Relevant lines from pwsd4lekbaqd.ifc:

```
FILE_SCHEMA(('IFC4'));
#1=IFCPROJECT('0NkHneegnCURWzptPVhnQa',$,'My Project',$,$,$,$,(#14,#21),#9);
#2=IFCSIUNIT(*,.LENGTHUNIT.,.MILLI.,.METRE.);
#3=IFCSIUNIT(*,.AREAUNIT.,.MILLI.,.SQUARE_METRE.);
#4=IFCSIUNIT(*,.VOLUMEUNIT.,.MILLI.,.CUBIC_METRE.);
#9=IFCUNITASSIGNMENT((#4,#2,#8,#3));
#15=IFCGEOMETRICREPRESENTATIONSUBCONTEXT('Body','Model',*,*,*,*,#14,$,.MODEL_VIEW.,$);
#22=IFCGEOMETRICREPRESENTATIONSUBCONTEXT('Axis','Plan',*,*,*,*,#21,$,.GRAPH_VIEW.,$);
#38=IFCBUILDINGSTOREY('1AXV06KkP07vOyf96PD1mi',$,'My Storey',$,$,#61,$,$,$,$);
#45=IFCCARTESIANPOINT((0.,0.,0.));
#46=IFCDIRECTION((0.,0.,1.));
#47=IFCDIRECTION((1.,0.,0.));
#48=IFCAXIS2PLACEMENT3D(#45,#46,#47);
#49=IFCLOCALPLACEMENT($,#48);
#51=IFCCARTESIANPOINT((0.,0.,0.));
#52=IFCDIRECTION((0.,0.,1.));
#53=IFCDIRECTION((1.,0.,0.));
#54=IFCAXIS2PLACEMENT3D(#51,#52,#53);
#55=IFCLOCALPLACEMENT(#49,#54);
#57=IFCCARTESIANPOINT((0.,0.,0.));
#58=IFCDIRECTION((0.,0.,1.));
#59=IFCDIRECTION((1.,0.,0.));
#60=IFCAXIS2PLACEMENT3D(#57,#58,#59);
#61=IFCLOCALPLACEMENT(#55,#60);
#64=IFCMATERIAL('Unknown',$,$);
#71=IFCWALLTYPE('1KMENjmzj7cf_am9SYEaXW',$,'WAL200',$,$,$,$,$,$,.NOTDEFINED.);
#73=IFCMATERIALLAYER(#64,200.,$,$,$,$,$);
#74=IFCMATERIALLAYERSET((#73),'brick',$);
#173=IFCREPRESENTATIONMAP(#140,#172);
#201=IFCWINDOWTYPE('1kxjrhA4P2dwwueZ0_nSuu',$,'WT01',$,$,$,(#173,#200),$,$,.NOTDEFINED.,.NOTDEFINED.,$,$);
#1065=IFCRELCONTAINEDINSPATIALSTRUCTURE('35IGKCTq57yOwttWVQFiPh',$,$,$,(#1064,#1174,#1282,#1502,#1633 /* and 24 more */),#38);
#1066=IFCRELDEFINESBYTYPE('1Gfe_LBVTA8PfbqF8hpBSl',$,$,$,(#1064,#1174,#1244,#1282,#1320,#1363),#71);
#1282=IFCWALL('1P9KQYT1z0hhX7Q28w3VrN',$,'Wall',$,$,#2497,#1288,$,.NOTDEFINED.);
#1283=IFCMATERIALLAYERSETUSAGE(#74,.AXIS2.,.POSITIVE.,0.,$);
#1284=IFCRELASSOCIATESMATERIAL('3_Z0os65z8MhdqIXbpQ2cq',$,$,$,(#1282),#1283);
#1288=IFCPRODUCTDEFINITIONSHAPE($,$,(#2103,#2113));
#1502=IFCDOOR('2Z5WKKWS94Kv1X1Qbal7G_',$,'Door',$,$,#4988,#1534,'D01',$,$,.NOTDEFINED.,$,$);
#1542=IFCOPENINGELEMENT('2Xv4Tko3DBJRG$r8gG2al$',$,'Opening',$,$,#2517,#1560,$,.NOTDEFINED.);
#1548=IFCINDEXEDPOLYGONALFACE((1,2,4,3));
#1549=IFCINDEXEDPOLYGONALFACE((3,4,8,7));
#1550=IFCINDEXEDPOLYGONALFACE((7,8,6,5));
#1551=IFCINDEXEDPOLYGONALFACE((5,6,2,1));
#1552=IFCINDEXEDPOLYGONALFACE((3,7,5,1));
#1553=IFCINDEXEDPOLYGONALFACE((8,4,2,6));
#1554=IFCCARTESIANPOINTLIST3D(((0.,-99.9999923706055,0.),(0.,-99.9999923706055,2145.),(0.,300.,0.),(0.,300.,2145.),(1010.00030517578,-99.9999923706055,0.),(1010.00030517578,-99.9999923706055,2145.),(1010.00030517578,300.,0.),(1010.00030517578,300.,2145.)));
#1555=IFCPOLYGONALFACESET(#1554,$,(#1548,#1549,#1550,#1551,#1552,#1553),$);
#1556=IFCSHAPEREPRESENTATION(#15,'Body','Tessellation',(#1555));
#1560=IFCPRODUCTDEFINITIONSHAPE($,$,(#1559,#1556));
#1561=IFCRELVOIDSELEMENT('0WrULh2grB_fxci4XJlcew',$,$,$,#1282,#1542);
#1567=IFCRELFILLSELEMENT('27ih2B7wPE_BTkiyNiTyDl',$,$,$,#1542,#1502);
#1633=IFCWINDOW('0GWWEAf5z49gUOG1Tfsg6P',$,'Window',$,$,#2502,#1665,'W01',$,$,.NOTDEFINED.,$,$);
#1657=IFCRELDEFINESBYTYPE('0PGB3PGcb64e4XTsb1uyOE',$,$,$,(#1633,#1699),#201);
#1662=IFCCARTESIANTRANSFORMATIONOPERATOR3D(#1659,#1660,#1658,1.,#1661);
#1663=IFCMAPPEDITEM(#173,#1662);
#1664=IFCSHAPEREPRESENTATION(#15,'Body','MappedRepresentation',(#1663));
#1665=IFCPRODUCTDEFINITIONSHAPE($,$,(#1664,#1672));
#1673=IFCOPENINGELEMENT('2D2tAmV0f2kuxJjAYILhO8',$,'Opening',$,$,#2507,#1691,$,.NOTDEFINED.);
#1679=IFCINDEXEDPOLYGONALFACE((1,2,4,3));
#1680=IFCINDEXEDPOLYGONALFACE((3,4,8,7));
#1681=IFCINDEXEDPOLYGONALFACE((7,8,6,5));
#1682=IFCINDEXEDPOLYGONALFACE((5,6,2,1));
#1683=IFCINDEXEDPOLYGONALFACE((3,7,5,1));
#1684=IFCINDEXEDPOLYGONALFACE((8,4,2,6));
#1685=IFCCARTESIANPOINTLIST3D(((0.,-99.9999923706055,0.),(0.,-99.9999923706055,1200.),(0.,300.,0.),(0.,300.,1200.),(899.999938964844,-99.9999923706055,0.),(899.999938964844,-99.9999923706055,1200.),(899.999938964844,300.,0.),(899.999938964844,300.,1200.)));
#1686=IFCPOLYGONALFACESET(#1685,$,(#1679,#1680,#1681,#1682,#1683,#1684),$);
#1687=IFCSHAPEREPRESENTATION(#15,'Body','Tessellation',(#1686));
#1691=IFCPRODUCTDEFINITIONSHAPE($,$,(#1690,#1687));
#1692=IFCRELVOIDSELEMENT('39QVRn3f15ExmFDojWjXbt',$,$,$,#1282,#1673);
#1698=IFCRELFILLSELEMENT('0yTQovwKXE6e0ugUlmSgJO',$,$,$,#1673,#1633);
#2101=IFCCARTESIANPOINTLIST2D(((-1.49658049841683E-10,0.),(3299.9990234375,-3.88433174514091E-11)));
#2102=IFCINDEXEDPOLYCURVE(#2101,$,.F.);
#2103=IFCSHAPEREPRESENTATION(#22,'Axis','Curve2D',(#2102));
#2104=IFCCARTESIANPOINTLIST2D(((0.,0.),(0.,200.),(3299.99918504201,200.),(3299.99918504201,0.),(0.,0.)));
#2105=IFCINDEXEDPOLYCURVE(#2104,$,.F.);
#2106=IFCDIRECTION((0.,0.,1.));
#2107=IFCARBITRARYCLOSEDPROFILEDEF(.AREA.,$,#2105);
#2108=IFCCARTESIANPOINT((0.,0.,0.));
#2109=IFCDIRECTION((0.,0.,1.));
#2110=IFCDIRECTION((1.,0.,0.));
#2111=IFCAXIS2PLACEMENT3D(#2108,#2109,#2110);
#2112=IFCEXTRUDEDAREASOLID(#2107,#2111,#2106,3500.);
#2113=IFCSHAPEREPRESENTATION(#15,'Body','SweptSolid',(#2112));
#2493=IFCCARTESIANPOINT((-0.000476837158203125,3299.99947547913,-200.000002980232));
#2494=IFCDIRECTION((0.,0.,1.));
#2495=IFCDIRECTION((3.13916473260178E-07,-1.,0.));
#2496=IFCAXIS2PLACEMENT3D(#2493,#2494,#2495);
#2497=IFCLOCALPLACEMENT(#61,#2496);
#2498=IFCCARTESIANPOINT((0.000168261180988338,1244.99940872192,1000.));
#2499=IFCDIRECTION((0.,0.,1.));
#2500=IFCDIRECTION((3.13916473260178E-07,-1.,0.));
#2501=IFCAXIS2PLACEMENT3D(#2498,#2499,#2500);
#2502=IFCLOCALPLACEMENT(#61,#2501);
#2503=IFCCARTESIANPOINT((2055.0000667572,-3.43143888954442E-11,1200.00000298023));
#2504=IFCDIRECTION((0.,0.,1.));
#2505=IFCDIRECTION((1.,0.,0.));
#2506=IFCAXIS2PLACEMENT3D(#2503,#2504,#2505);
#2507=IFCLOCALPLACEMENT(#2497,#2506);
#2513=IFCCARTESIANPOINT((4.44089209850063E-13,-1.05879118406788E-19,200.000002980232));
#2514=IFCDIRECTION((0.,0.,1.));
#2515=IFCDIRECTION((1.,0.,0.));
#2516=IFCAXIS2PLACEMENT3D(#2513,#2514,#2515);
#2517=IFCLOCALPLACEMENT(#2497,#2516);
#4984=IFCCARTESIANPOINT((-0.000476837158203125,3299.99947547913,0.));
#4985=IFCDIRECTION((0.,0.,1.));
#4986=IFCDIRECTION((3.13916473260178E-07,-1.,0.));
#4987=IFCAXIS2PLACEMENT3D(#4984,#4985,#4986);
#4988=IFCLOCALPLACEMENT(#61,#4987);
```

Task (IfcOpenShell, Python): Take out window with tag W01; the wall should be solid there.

```python
import ifcopenshell
import ifcopenshell.api.feature
import ifcopenshell.api.root
import ifcopenshell.geom
import ifcopenshell.util.shape

model = ifcopenshell.open("pwsd4lekbaqd.ifc")
settings = ifcopenshell.geom.settings()


def volume(element):
    """Net volume in cubic metres, openings subtracted."""
    shape = ifcopenshell.geom.create_shape(settings, element)
    return ifcopenshell.util.shape.get_volume(shape.geometry)


window = model.by_guid("0GWWEAf5z49gUOG1Tfsg6P")
opening = window.FillsVoids[0].RelatingOpeningElement
wall = opening.VoidsElements[0].RelatingBuildingElement
before = volume(wall)

ifcopenshell.api.root.remove_product(model, product=window)
ifcopenshell.api.feature.remove_feature(model, feature=opening)

after = volume(wall)

print(f"wall volume {before:.3f} -> {after:.3f} m3")

model.write("pwsd4lekbaqd_v2.ifc")
```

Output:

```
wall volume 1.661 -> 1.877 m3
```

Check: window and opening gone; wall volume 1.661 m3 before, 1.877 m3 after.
